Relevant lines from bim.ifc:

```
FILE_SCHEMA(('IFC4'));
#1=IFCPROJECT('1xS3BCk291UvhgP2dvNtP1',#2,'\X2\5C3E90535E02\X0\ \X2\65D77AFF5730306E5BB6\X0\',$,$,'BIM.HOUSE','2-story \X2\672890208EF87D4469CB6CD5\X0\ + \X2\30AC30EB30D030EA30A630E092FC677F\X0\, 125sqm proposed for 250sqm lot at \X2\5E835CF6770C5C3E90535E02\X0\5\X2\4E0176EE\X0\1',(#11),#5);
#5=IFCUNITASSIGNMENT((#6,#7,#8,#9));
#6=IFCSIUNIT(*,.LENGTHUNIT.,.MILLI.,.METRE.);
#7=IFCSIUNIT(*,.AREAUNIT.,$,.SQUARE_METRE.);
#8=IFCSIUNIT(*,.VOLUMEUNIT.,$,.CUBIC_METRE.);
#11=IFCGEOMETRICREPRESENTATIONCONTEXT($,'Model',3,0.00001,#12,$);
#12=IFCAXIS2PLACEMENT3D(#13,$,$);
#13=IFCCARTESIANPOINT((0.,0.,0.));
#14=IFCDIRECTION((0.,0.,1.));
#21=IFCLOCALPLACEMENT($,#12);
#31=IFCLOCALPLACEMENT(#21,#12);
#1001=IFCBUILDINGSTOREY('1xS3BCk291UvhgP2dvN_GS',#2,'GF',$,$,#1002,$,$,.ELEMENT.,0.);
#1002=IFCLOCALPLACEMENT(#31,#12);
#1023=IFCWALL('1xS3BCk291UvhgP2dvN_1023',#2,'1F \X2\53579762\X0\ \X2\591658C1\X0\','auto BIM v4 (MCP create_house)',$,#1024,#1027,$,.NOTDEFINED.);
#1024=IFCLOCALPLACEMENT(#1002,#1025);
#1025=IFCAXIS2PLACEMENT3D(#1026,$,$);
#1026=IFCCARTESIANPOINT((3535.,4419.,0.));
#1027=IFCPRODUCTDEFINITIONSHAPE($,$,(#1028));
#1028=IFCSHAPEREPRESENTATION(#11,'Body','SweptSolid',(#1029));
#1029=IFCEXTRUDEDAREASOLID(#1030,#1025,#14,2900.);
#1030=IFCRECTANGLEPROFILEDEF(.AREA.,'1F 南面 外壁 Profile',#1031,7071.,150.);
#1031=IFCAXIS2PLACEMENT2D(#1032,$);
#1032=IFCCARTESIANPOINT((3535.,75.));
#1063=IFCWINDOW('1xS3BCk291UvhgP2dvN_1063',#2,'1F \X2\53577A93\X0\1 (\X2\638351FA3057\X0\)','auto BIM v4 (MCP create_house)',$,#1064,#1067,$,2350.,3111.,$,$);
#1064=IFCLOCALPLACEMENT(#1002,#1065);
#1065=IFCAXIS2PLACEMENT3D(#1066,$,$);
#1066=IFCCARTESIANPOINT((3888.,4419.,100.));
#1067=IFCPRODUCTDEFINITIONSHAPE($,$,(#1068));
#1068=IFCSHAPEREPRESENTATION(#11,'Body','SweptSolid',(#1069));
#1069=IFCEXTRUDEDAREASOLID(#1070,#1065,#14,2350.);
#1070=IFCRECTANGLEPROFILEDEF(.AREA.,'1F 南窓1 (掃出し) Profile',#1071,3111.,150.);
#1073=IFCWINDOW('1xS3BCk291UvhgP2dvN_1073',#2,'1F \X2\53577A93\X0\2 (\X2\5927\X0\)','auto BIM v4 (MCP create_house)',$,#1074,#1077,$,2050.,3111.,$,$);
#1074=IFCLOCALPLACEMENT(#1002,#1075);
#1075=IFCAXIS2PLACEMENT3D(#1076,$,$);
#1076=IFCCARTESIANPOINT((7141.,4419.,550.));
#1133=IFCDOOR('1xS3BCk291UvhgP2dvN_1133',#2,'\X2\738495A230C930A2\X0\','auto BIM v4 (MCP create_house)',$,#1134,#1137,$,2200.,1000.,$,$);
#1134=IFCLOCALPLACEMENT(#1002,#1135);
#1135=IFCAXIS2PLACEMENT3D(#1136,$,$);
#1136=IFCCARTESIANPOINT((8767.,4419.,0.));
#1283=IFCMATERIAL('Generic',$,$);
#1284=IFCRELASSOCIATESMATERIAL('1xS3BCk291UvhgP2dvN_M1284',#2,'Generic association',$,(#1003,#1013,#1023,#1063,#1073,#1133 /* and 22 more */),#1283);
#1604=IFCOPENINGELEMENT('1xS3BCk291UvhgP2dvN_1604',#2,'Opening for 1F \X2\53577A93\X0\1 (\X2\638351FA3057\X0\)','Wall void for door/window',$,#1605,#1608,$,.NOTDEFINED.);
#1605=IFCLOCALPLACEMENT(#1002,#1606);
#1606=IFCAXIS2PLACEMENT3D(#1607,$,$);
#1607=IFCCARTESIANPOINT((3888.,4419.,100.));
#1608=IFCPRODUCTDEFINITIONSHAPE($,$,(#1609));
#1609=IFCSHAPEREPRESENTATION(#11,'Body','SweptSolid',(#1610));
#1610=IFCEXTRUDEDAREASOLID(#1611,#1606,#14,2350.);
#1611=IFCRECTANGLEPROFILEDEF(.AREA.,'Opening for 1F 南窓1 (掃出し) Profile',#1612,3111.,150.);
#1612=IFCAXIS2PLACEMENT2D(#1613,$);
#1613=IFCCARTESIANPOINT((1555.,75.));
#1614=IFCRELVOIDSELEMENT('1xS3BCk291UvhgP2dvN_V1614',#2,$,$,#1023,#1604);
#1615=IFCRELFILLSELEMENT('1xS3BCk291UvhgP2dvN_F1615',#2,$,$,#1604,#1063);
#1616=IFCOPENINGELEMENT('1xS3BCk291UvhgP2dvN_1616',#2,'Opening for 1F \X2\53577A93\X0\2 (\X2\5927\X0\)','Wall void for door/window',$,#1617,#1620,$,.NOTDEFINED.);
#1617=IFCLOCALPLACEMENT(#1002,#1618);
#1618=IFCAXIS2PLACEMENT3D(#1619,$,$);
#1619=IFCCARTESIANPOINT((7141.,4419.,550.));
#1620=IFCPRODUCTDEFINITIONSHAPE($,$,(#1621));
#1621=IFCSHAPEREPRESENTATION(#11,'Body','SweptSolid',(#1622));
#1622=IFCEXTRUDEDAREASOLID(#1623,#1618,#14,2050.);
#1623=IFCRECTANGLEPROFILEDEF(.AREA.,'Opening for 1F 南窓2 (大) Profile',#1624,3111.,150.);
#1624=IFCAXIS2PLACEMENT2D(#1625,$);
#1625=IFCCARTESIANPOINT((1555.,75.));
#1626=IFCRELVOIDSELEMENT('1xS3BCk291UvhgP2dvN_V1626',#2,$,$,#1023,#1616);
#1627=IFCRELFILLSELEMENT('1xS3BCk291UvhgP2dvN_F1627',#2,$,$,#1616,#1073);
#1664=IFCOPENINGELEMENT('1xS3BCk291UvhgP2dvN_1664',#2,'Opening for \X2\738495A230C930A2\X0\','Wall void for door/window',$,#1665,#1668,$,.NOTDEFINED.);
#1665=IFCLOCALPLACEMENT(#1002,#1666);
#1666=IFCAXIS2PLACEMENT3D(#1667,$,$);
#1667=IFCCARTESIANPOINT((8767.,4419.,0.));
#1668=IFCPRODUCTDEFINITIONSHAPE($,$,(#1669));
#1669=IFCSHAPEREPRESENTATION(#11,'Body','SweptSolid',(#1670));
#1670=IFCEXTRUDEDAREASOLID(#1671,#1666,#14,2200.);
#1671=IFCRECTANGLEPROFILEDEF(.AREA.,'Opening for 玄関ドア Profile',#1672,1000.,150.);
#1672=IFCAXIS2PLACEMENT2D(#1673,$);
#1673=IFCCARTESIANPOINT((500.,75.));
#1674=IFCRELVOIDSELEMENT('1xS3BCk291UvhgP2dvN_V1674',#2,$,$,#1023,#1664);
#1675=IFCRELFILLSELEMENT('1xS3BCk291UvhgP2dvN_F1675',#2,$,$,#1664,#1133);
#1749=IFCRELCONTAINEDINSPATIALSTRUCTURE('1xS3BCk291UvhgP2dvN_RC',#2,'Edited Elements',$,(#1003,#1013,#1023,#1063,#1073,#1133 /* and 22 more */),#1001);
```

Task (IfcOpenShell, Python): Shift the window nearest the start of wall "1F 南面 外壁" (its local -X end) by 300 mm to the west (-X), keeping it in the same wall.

```python
import ifcopenshell
import ifcopenshell.api.geometry
import ifcopenshell.util.placement
import ifcopenshell.util.unit

model = ifcopenshell.open("bim.ifc")
unit_scale = ifcopenshell.util.unit.calculate_unit_scale(model)

window = model.by_guid("1xS3BCk291UvhgP2dvN_1063")
opening = window.FillsVoids[0].RelatingOpeningElement
wall = opening.VoidsElements[0].RelatingBuildingElement

wall_matrix = ifcopenshell.util.placement.get_local_placement(wall.ObjectPlacement)
shift = wall_matrix[:3, 0] * -0.3 / unit_scale
before = ifcopenshell.util.placement.get_local_placement(window.ObjectPlacement)[:3, 3].copy()

# The window is not placed relative to its opening, so move both.
for product in (opening, window):
    matrix = ifcopenshell.util.placement.get_local_placement(product.ObjectPlacement)
    matrix[:3, 3] += shift
    ifcopenshell.api.geometry.edit_object_placement(model, product=product, matrix=matrix, is_si=False)

after = ifcopenshell.util.placement.get_local_placement(window.ObjectPlacement)[:3, 3]
print("window moved by", (after - before).round(3) + 0.0)

model.write("bim_edited.ifc")
```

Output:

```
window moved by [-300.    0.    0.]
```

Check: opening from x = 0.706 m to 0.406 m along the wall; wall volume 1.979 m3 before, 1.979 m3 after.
